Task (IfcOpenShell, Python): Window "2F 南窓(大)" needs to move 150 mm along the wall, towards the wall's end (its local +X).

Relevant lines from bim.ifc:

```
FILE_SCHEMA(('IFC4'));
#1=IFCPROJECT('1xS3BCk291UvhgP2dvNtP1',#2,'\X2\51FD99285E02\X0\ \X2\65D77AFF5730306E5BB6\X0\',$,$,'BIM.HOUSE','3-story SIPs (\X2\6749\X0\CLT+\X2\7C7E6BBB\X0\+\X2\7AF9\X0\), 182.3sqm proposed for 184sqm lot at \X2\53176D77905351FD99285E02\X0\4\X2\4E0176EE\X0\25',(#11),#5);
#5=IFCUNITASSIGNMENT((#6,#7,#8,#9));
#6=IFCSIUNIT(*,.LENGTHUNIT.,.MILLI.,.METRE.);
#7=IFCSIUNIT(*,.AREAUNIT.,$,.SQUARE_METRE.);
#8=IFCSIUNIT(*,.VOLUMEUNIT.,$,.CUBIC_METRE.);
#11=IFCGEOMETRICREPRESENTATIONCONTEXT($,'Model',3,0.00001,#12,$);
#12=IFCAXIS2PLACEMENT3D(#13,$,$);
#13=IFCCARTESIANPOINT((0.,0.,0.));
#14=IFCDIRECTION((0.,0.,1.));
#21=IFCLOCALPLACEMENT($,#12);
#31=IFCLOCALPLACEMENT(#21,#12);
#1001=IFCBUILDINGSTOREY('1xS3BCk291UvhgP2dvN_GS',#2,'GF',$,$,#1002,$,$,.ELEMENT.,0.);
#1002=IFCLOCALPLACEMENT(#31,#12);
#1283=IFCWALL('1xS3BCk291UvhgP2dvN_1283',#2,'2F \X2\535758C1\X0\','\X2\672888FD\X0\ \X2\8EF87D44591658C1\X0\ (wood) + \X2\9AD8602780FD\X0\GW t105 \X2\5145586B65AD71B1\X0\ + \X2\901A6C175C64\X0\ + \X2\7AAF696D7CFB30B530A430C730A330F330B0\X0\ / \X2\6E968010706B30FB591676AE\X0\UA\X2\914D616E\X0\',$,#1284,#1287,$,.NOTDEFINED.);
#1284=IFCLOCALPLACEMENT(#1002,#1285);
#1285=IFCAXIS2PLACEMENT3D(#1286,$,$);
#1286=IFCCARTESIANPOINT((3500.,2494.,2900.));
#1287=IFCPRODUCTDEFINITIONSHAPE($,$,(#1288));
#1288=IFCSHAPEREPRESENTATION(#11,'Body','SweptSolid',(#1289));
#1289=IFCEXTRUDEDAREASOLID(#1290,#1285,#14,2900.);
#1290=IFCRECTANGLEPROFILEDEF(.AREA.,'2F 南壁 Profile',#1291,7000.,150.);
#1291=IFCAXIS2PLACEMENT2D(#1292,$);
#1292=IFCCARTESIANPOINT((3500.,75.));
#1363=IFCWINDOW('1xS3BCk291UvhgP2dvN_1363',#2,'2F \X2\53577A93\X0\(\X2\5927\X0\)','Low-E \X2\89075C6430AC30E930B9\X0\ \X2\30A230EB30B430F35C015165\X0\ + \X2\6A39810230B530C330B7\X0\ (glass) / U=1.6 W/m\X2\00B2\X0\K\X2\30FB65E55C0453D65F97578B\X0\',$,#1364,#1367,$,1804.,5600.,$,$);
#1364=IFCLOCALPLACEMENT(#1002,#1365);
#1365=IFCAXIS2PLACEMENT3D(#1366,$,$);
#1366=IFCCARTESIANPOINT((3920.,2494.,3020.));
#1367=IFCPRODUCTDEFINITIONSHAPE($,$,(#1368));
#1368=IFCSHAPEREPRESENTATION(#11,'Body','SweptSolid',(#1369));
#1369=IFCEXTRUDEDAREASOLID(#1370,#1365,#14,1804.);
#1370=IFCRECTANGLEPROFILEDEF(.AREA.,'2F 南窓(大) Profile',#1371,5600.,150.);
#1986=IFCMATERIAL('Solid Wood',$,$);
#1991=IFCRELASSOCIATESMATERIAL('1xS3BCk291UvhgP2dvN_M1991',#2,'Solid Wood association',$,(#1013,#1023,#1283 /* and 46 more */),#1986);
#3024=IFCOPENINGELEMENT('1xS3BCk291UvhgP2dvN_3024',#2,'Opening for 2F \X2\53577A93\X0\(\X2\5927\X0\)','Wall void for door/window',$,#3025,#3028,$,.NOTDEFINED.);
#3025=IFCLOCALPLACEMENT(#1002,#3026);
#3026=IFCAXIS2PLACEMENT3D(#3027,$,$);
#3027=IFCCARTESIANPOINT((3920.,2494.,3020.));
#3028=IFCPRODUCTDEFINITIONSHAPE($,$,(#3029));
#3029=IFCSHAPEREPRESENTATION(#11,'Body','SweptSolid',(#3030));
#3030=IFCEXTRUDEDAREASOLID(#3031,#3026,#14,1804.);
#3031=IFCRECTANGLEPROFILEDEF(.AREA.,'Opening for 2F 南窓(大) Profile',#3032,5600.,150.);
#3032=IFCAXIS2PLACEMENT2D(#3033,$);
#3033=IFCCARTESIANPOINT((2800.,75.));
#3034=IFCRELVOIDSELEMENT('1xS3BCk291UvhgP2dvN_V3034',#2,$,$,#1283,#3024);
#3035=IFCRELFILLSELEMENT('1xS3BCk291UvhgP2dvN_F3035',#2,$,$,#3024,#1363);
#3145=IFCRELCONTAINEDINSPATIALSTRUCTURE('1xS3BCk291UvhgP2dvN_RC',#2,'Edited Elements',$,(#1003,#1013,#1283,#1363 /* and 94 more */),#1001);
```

```python
import ifcopenshell
import ifcopenshell.api.geometry
import ifcopenshell.util.placement

model = ifcopenshell.open("bim.ifc")

window = model.by_id(1363)
opening = window.FillsVoids[0].RelatingOpeningElement
wall = opening.VoidsElements[0].RelatingBuildingElement

wall_matrix = ifcopenshell.util.placement.get_local_placement(wall.ObjectPlacement)
shift = wall_matrix[:3, 0] * 150.0
before = ifcopenshell.util.placement.get_local_placement(window.ObjectPlacement)[:3, 3].copy()

# The window is not placed relative to its opening, so move both.
for product in (opening, window):
    matrix = ifcopenshell.util.placement.get_local_placement(product.ObjectPlacement)
    matrix[:3, 3] += shift
    ifcopenshell.api.geometry.edit_object_placement(model, product=product, matrix=matrix, is_si=False)

after = ifcopenshell.util.placement.get_local_placement(window.ObjectPlacement)[:3, 3]
print("window moved by", (after - before).round(3) + 0.0)

model.write("bim_rev.ifc")
```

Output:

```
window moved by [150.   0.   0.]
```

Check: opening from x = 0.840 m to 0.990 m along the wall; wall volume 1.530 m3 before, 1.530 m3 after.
